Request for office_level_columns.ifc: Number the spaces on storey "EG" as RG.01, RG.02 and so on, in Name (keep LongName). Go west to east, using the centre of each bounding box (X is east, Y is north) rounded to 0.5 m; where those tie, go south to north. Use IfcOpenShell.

First a look at what the model holds.

```python
import ifcopenshell
import ifcopenshell.util.element
import ifcopenshell.util.placement

model = ifcopenshell.open("office_level_columns.ifc")
print(model.schema)
storey = next(s for s in model.by_type("IfcBuildingStorey") if s.Name == "EG")
spaces = [e for e in ifcopenshell.util.element.get_decomposition(storey) if e.is_a("IfcSpace")]
for e in sorted(spaces, key=lambda e: e.id()):
    origin = ifcopenshell.util.placement.get_local_placement(e.ObjectPlacement)[:3, 3]
    print(e.id(), e.Name, e.LongName, origin.round(2) + 0.0, sep=" | ")
```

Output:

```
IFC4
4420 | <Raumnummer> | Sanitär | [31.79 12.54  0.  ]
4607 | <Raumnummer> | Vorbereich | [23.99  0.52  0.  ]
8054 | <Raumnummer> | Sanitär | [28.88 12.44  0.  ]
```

```python
import ifcopenshell
import ifcopenshell.geom
import ifcopenshell.util.element
import ifcopenshell.util.shape

model = ifcopenshell.open("office_level_columns.ifc")
settings = ifcopenshell.geom.settings()
settings.set("use-world-coords", True)


def centre(element):
    shape = ifcopenshell.geom.create_shape(settings, element)
    return ifcopenshell.util.shape.get_bbox_centroid(shape.geometry)


storey = next(s for s in model.by_type("IfcBuildingStorey") if s.Name == "EG")
spaces = [e for e in ifcopenshell.util.element.get_decomposition(storey) if e.is_a("IfcSpace")]

# Insertion points can sit at a corner or the storey origin, so sort by the geometry (in metres).
centres = {e: centre(e) for e in spaces}
spaces.sort(key=lambda e: (round(centres[e][0] / 0.5), centres[e][1]))

for i, e in enumerate(spaces, start=1):
    number = f"RG.{i:02d}"
    e.Name = number
    print(e.id(), number)

model.write("office_level_columns_updated.ifc")
```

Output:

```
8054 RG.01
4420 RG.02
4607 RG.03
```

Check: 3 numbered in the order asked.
